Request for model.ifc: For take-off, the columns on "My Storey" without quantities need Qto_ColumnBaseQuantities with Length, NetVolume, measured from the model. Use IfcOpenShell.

First a look at what the model holds.

```python
import ifcopenshell
import ifcopenshell.util.element
import ifcopenshell.util.unit

model = ifcopenshell.open("model.ifc")
print(model.schema)
for unit_type in ("LENGTHUNIT", "AREAUNIT", "VOLUMEUNIT"):
    print(unit_type, ifcopenshell.util.unit.calculate_unit_scale(model, unit_type))
storey = next(s for s in model.by_type("IfcBuildingStorey") if s.Name == "My Storey")
columns = [e for e in ifcopenshell.util.element.get_decomposition(storey) if e.is_a("IfcColumn")]
for e in sorted(columns, key=lambda e: e.id()):
    print(e.id(), e.is_a(), e.Name, list(ifcopenshell.util.element.get_psets(e, qtos_only=True)), sep=" | ")
```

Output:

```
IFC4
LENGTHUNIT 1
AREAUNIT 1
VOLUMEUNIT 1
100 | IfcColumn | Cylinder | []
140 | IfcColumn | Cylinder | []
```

```python
import ifcopenshell
import ifcopenshell.api.pset
import ifcopenshell.geom
import ifcopenshell.util.element
import ifcopenshell.util.shape
import ifcopenshell.util.unit

model = ifcopenshell.open("model.ifc")
unit_scale = ifcopenshell.util.unit.calculate_unit_scale(model)
volume_scale = ifcopenshell.util.unit.calculate_unit_scale(model, "VOLUMEUNIT")
settings = ifcopenshell.geom.settings()

storey = next(s for s in model.by_type("IfcBuildingStorey") if s.Name == "My Storey")
columns = [e for e in ifcopenshell.util.element.get_decomposition(storey) if e.is_a("IfcColumn")]

for e in sorted(columns, key=lambda e: e.id()):
    if ifcopenshell.util.element.get_psets(e, qtos_only=True, should_inherit=False):
        continue
    # Geometry comes back in metres, in the element's own axes.
    shape = ifcopenshell.geom.create_shape(settings, e)
    values = {
        "Length": ifcopenshell.util.shape.get_z(shape.geometry) / unit_scale,
        "NetVolume": ifcopenshell.util.shape.get_volume(shape.geometry) / volume_scale,
    }
    qto = ifcopenshell.api.pset.add_qto(model, product=e, name="Qto_ColumnBaseQuantities")
    ifcopenshell.api.pset.edit_qto(model, qto=qto, properties=values)
    print(e.id(), {k: round(v, 3) for k, v in values.items()})

model.write("model_v2.ifc")
```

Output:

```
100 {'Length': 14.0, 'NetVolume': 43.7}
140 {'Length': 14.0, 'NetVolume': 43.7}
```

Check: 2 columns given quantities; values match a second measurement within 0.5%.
